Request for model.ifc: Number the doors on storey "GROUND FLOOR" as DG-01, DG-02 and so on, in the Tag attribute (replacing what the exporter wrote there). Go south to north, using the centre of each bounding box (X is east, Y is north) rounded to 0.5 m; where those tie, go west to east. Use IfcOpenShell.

First a look at what the model holds.

```python
import ifcopenshell
import ifcopenshell.util.element
import ifcopenshell.util.placement

model = ifcopenshell.open("model.ifc")
print(model.schema)
storey = next(s for s in model.by_type("IfcBuildingStorey") if s.Name == "GROUND FLOOR")
doors = [e for e in ifcopenshell.util.element.get_decomposition(storey) if e.is_a("IfcDoor")]
for e in sorted(doors, key=lambda e: e.id()):
    origin = ifcopenshell.util.placement.get_local_placement(e.ObjectPlacement)[:3, 3]
    print(e.id(), e.Tag, e.Name, origin.round(2) + 0.0, sep=" | ")
```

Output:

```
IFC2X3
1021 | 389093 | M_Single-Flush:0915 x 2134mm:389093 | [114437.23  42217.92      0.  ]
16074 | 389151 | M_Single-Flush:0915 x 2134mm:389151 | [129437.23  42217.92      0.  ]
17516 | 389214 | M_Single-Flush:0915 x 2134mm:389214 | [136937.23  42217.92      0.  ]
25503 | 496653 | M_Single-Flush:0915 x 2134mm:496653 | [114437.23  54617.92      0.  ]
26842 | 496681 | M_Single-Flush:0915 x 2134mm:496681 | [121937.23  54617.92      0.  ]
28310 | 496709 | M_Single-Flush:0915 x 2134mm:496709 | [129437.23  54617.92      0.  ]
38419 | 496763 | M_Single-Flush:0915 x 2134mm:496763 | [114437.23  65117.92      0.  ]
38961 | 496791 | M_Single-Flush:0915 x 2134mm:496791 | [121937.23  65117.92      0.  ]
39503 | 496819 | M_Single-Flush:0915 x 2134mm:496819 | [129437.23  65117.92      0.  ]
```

```python
import ifcopenshell
import ifcopenshell.geom
import ifcopenshell.util.element
import ifcopenshell.util.shape

model = ifcopenshell.open("model.ifc")
settings = ifcopenshell.geom.settings()
settings.set("use-world-coords", True)


def centre(element):
    shape = ifcopenshell.geom.create_shape(settings, element)
    return ifcopenshell.util.shape.get_bbox_centroid(shape.geometry)


storey = next(s for s in model.by_type("IfcBuildingStorey") if s.Name == "GROUND FLOOR")
doors = [e for e in ifcopenshell.util.element.get_decomposition(storey) if e.is_a("IfcDoor")]

# Insertion points can sit at a corner or the storey origin, so sort by the geometry (in metres).
centres = {e: centre(e) for e in doors}
doors.sort(key=lambda e: (round(centres[e][1] / 0.5), centres[e][0]))

for i, e in enumerate(doors, start=1):
    number = f"DG-{i:02d}"
    e.Tag = number
    print(e.id(), number)

model.write("model_edited.ifc")
```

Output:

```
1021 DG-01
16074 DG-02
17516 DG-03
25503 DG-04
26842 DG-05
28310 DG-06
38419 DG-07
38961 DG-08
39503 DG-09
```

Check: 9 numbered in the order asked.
